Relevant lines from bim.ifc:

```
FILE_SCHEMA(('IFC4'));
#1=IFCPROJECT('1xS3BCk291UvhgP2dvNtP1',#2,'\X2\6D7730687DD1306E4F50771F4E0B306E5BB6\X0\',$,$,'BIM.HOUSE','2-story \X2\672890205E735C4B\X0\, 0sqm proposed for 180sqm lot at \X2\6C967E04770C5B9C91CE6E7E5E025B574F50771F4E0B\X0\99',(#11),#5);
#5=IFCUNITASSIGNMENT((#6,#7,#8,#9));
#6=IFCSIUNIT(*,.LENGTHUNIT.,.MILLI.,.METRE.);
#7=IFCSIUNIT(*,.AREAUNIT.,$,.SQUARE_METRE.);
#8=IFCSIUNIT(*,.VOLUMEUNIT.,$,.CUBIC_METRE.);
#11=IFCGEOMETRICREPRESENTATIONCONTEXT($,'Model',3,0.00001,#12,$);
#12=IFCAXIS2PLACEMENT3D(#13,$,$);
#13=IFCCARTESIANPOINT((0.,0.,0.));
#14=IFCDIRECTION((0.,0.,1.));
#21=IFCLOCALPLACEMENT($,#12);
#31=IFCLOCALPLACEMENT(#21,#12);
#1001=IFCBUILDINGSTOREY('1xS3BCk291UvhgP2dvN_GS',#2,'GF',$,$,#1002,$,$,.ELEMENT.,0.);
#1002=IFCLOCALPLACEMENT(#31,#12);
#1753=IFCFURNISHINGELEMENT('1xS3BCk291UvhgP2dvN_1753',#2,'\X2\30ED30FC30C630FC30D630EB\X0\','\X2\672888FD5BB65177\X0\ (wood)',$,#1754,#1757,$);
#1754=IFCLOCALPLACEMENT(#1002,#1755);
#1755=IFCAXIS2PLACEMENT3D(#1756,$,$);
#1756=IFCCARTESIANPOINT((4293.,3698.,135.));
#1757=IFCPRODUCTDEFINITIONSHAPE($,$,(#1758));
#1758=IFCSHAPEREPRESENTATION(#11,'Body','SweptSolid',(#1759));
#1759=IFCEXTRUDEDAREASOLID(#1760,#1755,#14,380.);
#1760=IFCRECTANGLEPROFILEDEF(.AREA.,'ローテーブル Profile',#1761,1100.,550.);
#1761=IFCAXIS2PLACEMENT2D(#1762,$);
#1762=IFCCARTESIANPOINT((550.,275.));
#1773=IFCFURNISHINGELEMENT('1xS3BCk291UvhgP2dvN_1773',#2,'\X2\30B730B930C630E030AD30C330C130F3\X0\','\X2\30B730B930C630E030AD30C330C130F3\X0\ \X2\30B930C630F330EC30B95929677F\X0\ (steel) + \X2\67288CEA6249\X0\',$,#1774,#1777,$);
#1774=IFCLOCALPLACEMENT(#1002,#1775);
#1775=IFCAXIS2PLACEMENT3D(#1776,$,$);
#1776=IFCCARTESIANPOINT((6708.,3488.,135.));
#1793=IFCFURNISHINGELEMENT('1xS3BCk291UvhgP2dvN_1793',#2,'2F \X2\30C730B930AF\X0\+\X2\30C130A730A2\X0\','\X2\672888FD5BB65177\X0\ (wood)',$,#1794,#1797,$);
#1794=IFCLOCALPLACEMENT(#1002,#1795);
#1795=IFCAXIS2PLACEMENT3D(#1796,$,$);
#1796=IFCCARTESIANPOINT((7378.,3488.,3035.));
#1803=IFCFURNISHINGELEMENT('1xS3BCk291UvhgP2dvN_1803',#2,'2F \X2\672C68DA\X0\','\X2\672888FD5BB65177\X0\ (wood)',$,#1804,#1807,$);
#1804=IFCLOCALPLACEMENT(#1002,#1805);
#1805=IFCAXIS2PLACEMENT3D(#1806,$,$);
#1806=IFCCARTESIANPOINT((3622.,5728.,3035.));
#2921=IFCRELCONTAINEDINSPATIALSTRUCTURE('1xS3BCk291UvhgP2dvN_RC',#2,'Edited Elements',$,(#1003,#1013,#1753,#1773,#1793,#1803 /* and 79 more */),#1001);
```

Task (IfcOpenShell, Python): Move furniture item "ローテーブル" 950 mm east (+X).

```python
import ifcopenshell
import ifcopenshell.api.geometry
import ifcopenshell.util.placement

model = ifcopenshell.open("bim.ifc")

item = model.by_guid("1xS3BCk291UvhgP2dvN_1753")
matrix = ifcopenshell.util.placement.get_local_placement(item.ObjectPlacement)
matrix[0, 3] += 950.0
ifcopenshell.api.geometry.edit_object_placement(model, product=item, matrix=matrix, is_si=False)

print(ifcopenshell.util.placement.get_local_placement(item.ObjectPlacement).round(3) + 0.0)

model.write("bim_rev.ifc")
```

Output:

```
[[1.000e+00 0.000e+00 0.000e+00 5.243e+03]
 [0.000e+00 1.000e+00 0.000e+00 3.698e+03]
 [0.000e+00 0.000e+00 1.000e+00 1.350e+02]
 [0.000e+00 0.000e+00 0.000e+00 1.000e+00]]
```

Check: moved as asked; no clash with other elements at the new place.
